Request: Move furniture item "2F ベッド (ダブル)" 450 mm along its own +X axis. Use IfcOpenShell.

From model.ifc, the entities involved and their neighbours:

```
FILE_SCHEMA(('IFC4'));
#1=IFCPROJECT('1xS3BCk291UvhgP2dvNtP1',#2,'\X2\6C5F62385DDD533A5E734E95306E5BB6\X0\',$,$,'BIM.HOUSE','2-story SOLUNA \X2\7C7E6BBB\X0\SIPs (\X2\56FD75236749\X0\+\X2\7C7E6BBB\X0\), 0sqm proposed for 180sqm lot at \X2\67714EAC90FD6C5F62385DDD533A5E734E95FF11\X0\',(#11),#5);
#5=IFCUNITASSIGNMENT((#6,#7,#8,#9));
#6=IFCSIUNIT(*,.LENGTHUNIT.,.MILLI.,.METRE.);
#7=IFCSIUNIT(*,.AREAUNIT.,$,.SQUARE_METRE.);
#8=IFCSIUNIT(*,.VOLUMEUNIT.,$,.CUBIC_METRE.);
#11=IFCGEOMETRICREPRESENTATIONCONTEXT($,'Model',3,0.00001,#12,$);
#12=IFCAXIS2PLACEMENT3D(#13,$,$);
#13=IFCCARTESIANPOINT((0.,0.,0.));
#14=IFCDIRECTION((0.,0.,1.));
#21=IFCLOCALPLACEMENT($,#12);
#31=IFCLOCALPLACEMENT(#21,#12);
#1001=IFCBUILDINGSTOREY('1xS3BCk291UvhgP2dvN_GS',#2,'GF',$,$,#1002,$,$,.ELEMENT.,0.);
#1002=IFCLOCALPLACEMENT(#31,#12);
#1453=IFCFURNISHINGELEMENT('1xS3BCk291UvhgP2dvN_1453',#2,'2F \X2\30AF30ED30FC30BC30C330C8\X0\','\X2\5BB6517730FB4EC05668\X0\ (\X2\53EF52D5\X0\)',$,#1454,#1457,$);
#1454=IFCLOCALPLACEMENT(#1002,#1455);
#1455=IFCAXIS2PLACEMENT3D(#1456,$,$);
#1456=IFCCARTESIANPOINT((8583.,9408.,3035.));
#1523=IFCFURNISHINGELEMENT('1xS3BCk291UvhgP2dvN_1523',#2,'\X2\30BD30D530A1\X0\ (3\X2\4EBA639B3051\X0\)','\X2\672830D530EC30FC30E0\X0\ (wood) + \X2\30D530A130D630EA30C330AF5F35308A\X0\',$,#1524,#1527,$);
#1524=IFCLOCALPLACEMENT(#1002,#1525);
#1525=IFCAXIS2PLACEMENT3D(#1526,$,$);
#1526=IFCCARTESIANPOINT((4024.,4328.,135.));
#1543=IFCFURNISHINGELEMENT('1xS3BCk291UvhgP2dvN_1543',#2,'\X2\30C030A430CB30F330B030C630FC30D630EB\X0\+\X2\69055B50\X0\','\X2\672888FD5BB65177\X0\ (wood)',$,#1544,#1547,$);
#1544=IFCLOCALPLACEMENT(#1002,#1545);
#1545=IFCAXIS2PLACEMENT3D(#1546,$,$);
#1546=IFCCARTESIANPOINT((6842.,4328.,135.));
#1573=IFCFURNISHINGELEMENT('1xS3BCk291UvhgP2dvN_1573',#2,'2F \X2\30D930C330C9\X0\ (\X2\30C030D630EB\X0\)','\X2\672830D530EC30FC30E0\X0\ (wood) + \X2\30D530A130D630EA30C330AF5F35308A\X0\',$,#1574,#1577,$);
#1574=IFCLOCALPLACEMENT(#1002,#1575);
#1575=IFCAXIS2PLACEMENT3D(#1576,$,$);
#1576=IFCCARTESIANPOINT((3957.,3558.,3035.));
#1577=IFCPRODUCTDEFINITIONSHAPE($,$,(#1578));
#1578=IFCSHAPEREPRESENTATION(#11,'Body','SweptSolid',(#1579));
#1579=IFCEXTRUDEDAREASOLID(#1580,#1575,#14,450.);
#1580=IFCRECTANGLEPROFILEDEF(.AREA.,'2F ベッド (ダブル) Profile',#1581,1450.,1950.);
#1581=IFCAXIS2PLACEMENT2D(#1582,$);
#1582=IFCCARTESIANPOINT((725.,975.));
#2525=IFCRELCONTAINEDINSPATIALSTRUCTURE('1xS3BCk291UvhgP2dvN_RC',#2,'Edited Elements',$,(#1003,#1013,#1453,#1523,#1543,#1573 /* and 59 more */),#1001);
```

```python
import ifcopenshell
import ifcopenshell.api.geometry
import ifcopenshell.util.placement
import ifcopenshell.util.unit

model = ifcopenshell.open("model.ifc")
unit_scale = ifcopenshell.util.unit.calculate_unit_scale(model)

item = model.by_guid("1xS3BCk291UvhgP2dvN_1573")
matrix = ifcopenshell.util.placement.get_local_placement(item.ObjectPlacement)
matrix[:3, 3] += matrix[:3, 0] * 0.45 / unit_scale
ifcopenshell.api.geometry.edit_object_placement(model, product=item, matrix=matrix, is_si=False)

print(ifcopenshell.util.placement.get_local_placement(item.ObjectPlacement).round(3) + 0.0)

model.write("model_updated.ifc")
```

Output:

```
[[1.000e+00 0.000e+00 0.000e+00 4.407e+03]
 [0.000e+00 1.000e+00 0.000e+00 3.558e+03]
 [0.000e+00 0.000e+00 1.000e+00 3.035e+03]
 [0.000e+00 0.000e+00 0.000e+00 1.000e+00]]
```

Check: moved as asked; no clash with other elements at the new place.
